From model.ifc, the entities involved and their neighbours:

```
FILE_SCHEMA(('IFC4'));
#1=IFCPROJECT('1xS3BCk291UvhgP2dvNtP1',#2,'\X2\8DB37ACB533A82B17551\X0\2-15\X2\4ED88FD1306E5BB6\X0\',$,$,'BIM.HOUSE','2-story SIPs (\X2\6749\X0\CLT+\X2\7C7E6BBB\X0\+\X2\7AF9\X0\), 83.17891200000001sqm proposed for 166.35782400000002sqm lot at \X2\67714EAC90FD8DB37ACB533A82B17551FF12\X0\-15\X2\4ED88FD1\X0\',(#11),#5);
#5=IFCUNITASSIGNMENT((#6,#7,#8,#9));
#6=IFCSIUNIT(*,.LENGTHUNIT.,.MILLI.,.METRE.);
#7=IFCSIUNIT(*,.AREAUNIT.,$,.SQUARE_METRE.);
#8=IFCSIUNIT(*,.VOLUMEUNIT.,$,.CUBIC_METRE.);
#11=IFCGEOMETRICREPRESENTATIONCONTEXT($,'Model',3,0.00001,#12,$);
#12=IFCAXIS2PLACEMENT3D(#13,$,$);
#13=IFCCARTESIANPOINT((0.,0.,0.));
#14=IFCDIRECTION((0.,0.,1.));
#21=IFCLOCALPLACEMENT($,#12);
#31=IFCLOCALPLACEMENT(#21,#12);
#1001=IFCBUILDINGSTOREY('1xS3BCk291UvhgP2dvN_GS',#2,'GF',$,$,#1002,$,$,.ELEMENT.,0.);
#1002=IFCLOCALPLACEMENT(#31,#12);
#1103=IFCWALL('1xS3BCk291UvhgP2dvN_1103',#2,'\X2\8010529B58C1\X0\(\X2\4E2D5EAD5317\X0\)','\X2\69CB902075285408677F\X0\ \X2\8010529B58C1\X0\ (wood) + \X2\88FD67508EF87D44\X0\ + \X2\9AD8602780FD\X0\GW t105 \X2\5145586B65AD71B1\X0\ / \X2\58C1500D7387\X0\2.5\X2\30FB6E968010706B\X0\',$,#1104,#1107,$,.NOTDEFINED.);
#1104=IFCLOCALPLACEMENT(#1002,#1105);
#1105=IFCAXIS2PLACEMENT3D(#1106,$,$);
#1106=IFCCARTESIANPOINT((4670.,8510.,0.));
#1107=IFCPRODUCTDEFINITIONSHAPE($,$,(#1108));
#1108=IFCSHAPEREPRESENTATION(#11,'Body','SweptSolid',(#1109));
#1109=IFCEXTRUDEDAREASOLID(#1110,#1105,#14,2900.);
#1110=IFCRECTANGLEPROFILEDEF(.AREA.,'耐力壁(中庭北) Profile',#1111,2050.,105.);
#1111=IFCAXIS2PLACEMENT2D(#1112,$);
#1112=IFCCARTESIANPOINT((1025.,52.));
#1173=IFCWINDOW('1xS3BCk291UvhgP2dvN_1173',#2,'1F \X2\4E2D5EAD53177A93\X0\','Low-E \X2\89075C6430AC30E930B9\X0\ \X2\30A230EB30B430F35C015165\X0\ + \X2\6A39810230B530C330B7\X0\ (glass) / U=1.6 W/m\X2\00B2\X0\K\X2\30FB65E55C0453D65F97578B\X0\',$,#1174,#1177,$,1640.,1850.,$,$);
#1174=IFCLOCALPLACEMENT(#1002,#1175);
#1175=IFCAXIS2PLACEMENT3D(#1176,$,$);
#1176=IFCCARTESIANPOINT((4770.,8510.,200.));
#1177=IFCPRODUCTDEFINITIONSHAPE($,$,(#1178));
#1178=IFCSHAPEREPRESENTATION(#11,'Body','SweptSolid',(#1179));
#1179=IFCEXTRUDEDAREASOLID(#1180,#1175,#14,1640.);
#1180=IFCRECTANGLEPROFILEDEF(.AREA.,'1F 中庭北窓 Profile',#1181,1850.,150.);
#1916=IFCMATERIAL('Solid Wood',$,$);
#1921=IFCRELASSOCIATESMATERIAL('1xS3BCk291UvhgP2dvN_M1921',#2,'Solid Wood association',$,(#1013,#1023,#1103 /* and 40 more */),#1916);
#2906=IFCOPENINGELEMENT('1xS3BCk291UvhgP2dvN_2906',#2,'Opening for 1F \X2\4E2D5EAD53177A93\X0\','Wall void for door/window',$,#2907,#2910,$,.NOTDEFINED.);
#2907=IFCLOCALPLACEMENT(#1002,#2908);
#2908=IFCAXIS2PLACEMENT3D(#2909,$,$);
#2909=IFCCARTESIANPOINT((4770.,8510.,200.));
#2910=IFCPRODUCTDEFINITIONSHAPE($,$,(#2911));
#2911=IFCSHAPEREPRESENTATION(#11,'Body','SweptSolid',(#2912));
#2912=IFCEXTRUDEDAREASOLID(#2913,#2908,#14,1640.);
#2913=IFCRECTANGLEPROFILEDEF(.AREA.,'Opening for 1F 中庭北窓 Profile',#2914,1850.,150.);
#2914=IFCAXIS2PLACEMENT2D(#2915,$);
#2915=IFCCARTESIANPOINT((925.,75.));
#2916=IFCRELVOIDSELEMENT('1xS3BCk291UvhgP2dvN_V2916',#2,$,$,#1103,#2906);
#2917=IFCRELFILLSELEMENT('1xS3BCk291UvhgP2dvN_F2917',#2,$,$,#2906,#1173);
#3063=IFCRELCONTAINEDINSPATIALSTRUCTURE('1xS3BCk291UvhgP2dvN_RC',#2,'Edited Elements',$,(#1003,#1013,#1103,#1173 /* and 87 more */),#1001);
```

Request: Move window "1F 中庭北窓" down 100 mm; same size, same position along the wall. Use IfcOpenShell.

```python
import numpy as np
import ifcopenshell
import ifcopenshell.api.geometry
import ifcopenshell.util.placement
import ifcopenshell.util.unit

model = ifcopenshell.open("model.ifc")
unit_scale = ifcopenshell.util.unit.calculate_unit_scale(model)

window = model.by_id(1173)
opening = window.FillsVoids[0].RelatingOpeningElement
dz = -0.1 / unit_scale

shift = np.array([0.0, 0.0, dz])
# The window is not placed relative to its opening, so move both.
for product in (opening, window):
    matrix = ifcopenshell.util.placement.get_local_placement(product.ObjectPlacement)
    matrix[:3, 3] += shift
    ifcopenshell.api.geometry.edit_object_placement(model, product=product, matrix=matrix, is_si=False)

print(f"moved by {dz * unit_scale:+.3f} m")

model.write("model_rev.ifc")
```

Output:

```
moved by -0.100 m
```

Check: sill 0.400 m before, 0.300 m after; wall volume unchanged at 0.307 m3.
